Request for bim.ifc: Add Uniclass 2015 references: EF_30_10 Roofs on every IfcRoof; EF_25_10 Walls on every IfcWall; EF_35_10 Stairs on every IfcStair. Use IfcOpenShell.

First a look at what the model holds.

```python
import ifcopenshell

model = ifcopenshell.open("bim.ifc")
print(model.schema)
print("classifications:", [c.Name for c in model.by_type("IfcClassification")])
for ifc_class in ("IfcDoor", "IfcRoof", "IfcStair", "IfcWall", "IfcWindow"):
    print(ifc_class, len(model.by_type(ifc_class)))
```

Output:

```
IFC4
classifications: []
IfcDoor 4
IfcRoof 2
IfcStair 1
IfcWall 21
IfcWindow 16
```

```python
import ifcopenshell
import ifcopenshell.api.classification

model = ifcopenshell.open("bim.ifc")

system = ifcopenshell.api.classification.add_classification(model, classification="Uniclass 2015")

codes = {
    "IfcRoof": ("EF_30_10", "Roofs"),
    "IfcWall": ("EF_25_10", "Walls"),
    "IfcStair": ("EF_35_10", "Stairs"),
}
for ifc_class, (code, name) in codes.items():
    products = model.by_type(ifc_class)
    ifcopenshell.api.classification.add_reference(
        model, products=products, classification=system, identification=code, name=name
    )
    print(code, len(products))

model.write("bim_updated.ifc")
```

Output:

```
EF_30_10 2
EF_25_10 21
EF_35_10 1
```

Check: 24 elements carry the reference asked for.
